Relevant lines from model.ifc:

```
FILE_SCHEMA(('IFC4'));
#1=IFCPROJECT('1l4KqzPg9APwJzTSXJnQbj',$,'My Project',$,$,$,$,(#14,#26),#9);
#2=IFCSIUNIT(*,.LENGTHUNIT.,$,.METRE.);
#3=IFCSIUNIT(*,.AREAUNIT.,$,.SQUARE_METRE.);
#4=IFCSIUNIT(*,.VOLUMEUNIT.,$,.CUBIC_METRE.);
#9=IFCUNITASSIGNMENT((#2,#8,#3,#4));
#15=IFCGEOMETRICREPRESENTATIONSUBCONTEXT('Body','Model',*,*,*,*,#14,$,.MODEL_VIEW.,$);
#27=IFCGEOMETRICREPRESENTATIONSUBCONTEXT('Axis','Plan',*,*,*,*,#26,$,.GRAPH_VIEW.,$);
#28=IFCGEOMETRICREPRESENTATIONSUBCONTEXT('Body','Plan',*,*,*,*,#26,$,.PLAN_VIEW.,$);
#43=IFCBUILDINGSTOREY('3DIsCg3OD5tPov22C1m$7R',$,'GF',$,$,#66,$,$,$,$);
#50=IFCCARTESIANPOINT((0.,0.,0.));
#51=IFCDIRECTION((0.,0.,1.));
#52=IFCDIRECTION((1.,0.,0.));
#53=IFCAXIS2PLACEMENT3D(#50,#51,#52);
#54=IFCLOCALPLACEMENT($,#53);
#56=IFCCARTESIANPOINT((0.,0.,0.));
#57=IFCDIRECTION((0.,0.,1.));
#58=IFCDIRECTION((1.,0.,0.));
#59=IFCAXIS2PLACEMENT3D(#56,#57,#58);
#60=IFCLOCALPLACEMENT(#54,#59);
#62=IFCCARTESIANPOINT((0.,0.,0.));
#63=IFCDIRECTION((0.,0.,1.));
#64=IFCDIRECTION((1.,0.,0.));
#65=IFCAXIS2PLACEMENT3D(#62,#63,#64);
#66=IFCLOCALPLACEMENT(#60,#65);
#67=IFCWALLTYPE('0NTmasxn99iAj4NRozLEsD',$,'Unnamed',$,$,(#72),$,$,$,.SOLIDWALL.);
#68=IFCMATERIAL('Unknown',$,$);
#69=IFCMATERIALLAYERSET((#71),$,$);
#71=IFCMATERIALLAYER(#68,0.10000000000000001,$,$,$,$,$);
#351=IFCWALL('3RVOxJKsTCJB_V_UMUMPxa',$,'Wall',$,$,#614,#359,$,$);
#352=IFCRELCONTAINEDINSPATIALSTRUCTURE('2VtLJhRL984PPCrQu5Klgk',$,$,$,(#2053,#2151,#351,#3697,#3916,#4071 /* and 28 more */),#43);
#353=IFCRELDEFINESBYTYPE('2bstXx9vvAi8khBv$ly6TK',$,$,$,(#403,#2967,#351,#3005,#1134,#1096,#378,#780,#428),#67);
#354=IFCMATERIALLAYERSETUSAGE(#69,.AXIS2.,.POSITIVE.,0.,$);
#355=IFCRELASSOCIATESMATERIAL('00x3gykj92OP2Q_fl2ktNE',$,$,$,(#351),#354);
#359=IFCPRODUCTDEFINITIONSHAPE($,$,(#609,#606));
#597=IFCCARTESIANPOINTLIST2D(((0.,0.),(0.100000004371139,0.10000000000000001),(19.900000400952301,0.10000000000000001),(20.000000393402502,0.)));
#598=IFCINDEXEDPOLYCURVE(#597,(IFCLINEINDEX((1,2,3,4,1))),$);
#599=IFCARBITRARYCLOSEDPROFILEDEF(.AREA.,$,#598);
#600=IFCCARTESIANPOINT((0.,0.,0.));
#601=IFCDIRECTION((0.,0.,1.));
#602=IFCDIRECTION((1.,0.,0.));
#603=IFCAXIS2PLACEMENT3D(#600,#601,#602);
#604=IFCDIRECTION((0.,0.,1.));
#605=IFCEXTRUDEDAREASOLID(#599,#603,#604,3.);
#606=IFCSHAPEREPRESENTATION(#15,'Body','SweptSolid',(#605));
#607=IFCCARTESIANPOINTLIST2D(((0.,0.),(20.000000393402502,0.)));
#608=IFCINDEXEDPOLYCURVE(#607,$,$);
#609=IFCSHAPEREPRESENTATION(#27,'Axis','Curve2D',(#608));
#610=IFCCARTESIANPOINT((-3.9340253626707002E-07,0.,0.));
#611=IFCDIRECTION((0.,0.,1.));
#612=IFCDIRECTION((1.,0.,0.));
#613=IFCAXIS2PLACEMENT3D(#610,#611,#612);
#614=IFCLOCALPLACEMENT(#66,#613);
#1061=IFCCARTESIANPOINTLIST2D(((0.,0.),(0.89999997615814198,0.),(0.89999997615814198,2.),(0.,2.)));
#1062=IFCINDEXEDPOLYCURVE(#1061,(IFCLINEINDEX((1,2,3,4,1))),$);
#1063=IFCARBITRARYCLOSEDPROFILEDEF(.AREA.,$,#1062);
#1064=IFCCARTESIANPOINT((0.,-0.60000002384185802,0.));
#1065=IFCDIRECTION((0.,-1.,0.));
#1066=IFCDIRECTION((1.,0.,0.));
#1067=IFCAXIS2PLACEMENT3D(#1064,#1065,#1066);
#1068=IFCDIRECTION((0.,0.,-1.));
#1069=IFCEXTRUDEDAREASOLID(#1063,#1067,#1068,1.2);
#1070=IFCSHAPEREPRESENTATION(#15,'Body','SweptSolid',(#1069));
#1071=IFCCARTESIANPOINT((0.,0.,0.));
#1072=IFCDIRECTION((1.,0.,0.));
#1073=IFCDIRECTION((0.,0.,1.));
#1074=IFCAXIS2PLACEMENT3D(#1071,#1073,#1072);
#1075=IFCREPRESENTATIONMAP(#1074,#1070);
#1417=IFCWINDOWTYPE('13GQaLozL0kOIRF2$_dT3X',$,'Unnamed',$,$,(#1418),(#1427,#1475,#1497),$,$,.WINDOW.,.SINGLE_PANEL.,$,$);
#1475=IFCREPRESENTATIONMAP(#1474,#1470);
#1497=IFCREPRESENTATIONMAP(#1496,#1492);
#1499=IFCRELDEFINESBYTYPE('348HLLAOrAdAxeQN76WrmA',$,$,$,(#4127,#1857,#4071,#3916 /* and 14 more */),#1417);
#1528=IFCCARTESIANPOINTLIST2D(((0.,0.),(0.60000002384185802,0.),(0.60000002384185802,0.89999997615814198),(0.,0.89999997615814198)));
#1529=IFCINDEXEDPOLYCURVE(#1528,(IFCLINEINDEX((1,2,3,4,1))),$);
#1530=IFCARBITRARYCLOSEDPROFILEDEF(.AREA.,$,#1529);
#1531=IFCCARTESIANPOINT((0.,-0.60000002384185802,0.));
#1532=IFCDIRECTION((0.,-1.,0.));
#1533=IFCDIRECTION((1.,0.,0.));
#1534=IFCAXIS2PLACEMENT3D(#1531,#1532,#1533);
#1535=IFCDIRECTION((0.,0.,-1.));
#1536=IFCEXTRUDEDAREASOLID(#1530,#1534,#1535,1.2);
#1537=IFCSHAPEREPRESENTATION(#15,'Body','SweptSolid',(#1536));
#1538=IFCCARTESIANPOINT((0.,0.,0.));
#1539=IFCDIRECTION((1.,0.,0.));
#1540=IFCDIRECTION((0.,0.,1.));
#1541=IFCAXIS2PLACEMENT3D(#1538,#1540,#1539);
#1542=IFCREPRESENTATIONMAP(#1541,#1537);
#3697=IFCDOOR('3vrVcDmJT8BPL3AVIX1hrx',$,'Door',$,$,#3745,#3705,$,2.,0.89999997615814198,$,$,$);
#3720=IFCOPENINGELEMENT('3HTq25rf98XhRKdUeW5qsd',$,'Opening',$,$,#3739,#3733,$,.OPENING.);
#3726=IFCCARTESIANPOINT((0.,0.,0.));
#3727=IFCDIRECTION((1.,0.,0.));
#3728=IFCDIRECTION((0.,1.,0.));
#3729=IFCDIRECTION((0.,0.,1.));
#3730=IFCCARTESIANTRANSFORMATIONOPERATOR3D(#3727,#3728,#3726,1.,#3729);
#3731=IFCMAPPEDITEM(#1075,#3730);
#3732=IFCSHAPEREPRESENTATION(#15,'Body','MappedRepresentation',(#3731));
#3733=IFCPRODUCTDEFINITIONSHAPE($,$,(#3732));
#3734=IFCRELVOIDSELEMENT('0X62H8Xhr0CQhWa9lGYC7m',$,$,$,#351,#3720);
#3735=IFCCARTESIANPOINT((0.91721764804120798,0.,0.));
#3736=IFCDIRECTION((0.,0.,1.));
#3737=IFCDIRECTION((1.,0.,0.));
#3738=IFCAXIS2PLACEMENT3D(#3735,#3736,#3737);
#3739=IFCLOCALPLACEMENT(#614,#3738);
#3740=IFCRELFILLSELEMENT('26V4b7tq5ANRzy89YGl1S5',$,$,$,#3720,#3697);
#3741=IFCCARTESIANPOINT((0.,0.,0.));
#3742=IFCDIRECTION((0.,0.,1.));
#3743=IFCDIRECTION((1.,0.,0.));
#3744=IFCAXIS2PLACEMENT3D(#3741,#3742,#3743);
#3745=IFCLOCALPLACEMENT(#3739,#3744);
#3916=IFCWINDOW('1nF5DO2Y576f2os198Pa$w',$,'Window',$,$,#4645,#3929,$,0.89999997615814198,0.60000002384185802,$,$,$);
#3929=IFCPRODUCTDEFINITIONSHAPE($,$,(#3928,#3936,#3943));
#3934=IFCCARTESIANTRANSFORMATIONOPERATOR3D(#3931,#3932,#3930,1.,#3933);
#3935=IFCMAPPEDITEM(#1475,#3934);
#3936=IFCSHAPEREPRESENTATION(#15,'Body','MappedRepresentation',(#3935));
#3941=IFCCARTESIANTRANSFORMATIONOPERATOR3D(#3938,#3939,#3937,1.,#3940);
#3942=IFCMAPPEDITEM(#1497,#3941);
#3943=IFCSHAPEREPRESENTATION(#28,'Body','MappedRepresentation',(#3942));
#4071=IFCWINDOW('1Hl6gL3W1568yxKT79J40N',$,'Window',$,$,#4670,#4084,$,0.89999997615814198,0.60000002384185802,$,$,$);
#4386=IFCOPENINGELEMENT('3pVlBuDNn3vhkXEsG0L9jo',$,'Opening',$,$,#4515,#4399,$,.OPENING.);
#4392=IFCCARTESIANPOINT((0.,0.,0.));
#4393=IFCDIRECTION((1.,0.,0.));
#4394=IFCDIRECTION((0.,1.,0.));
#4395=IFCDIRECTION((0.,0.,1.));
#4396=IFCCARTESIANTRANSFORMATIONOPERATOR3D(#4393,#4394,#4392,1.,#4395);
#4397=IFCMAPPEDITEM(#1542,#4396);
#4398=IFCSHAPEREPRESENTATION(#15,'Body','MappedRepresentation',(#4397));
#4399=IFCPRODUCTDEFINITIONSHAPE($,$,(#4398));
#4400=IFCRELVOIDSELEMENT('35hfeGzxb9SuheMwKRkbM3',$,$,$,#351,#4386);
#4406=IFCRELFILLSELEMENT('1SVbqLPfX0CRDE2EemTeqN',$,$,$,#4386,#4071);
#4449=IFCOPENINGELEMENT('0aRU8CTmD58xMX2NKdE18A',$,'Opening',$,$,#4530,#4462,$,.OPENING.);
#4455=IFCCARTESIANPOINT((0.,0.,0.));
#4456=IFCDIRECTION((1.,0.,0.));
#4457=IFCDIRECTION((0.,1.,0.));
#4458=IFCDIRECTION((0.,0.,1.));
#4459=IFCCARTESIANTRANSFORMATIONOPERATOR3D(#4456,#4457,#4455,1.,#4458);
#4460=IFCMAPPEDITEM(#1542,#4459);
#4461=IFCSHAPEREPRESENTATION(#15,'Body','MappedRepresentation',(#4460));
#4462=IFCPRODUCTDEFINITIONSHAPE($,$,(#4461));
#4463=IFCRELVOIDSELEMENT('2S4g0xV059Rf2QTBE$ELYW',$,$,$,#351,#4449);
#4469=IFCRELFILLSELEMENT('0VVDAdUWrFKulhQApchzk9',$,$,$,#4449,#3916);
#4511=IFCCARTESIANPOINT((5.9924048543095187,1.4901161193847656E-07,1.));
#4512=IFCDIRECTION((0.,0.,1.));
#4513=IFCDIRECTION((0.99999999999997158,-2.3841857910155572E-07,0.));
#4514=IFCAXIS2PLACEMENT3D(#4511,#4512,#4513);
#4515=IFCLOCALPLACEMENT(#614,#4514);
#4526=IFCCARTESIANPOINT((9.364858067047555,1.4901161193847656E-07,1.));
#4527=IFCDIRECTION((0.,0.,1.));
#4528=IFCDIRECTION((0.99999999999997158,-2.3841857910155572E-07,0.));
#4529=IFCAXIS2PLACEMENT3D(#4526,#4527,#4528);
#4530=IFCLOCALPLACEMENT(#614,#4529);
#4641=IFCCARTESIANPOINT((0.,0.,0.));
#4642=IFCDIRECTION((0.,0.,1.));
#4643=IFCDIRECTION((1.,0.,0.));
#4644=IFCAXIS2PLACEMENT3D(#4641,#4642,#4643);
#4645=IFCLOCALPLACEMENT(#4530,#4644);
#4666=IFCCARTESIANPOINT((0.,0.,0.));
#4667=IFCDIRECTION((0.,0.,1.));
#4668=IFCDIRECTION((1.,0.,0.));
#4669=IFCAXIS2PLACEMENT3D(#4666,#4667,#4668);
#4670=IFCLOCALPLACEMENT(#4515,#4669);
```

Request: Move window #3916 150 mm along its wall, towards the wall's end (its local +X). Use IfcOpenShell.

```python
import ifcopenshell
import ifcopenshell.api.geometry
import ifcopenshell.util.placement
import ifcopenshell.util.unit

model = ifcopenshell.open("model.ifc")
unit_scale = ifcopenshell.util.unit.calculate_unit_scale(model)

window = model.by_guid("1nF5DO2Y576f2os198Pa$w")
opening = window.FillsVoids[0].RelatingOpeningElement
wall = opening.VoidsElements[0].RelatingBuildingElement

wall_matrix = ifcopenshell.util.placement.get_local_placement(wall.ObjectPlacement)
shift = wall_matrix[:3, 0] * 0.15 / unit_scale
before = ifcopenshell.util.placement.get_local_placement(window.ObjectPlacement)[:3, 3].copy()

# The window is placed relative to its opening, so it follows when the opening moves.
matrix = ifcopenshell.util.placement.get_local_placement(opening.ObjectPlacement)
matrix[:3, 3] += shift
ifcopenshell.api.geometry.edit_object_placement(
    model, product=opening, matrix=matrix, is_si=False, should_transform_children=True
)

after = ifcopenshell.util.placement.get_local_placement(window.ObjectPlacement)[:3, 3]
print("window moved by", (after - before).round(3) + 0.0)

model.write("model_edited.ifc")
```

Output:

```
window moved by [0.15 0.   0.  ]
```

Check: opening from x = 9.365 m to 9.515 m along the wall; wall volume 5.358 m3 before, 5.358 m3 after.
